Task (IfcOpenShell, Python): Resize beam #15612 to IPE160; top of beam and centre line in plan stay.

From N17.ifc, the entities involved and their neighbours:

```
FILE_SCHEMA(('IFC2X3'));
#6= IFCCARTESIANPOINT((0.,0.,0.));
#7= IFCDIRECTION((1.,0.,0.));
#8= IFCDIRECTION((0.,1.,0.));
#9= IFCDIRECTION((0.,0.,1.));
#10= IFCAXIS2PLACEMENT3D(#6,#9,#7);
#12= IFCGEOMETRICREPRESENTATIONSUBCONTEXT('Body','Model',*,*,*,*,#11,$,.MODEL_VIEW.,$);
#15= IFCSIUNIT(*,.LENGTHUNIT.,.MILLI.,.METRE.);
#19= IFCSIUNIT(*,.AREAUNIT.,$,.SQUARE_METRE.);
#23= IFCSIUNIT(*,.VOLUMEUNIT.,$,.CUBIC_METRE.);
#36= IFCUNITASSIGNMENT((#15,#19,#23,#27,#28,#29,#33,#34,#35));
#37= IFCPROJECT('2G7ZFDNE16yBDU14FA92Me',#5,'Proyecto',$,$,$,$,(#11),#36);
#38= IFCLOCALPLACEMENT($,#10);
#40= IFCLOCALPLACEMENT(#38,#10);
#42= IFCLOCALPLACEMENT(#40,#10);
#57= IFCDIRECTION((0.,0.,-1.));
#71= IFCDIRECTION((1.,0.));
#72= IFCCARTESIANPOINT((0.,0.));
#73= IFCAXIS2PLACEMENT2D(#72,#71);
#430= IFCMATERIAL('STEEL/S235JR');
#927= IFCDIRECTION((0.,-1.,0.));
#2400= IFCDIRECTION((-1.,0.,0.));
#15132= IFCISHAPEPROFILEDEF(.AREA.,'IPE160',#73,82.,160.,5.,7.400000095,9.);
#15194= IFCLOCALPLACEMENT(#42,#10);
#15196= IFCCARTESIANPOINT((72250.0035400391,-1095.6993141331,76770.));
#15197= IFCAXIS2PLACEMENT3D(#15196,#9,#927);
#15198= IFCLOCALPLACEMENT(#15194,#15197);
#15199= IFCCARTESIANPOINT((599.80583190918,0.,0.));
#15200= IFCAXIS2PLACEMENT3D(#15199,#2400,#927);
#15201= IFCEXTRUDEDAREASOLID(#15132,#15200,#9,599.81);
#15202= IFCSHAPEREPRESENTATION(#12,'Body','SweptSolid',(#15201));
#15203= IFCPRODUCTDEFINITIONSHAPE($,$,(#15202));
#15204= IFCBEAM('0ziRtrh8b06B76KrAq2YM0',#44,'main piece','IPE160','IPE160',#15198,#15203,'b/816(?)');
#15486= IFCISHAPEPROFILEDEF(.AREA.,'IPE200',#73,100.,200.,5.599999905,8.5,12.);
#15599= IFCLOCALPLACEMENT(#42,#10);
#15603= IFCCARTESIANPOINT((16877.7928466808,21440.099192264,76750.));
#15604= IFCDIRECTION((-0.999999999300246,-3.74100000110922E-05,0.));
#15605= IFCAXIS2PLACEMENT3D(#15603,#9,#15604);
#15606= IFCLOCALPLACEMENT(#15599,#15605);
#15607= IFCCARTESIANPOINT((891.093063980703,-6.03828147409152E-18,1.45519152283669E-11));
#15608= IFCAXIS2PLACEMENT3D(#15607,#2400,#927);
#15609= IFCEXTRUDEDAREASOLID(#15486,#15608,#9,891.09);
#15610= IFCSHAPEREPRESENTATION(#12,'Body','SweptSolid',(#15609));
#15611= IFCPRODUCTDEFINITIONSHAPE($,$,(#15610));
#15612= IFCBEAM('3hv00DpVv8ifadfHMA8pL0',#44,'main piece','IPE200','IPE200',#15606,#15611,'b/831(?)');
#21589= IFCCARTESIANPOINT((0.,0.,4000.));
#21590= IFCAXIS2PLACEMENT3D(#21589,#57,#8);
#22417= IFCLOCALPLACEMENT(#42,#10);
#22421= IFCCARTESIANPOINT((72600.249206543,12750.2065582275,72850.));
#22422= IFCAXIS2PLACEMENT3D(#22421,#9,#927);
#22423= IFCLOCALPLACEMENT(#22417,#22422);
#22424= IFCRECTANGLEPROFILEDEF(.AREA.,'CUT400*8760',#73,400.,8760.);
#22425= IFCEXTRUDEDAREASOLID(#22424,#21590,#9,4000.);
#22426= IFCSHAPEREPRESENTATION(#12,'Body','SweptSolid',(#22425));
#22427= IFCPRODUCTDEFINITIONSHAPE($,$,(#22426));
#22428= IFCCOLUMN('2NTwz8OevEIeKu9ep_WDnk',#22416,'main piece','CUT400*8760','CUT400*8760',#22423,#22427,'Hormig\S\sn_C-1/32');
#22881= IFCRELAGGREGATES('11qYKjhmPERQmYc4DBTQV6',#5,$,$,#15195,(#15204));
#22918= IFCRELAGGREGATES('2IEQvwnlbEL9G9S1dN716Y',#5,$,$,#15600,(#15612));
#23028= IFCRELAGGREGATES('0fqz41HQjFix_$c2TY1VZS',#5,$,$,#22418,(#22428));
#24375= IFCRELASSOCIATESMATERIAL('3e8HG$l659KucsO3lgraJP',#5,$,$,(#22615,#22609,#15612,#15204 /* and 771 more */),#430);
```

```python
import ifcopenshell
import ifcopenshell.util.element
import ifcopenshell.util.representation

model = ifcopenshell.open("N17.ifc")

member = model.by_id(15612)
source = next(p for p in model.by_type("IfcIShapeProfileDef") if p.ProfileName == "IPE160")

body = ifcopenshell.util.representation.get_representation(member, "Model", "Body")
solid = body.Items[0]
old_profile = solid.SweptArea

# Copy the section's sizes but keep this member's own profile position.
profile = ifcopenshell.util.element.copy(model, source)
# Profiles are centred, so shift by half the change in depth to hold the top.
shift = (old_profile.OverallDepth - profile.OverallDepth) / 2
x, y = old_profile.Position.Location.Coordinates
up = (0.0, 1.0)  # upwards, in the solid's own plane
location = model.createIfcCartesianPoint((x + up[0] * shift, y + up[1] * shift))
profile.Position = model.createIfcAxis2Placement2D(location, old_profile.Position.RefDirection)
solid.SweptArea = profile
if not model.get_total_inverses(old_profile):
    ifcopenshell.util.element.remove_deep2(model, old_profile)
member.Description = member.Description.replace("IPE200", "IPE160")
member.ObjectType = member.ObjectType.replace("IPE200", "IPE160")

print(solid.SweptArea)

model.write("N17_edited.ifc")
```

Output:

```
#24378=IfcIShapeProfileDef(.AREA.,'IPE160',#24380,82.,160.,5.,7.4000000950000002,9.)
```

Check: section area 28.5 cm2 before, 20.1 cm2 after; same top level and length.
